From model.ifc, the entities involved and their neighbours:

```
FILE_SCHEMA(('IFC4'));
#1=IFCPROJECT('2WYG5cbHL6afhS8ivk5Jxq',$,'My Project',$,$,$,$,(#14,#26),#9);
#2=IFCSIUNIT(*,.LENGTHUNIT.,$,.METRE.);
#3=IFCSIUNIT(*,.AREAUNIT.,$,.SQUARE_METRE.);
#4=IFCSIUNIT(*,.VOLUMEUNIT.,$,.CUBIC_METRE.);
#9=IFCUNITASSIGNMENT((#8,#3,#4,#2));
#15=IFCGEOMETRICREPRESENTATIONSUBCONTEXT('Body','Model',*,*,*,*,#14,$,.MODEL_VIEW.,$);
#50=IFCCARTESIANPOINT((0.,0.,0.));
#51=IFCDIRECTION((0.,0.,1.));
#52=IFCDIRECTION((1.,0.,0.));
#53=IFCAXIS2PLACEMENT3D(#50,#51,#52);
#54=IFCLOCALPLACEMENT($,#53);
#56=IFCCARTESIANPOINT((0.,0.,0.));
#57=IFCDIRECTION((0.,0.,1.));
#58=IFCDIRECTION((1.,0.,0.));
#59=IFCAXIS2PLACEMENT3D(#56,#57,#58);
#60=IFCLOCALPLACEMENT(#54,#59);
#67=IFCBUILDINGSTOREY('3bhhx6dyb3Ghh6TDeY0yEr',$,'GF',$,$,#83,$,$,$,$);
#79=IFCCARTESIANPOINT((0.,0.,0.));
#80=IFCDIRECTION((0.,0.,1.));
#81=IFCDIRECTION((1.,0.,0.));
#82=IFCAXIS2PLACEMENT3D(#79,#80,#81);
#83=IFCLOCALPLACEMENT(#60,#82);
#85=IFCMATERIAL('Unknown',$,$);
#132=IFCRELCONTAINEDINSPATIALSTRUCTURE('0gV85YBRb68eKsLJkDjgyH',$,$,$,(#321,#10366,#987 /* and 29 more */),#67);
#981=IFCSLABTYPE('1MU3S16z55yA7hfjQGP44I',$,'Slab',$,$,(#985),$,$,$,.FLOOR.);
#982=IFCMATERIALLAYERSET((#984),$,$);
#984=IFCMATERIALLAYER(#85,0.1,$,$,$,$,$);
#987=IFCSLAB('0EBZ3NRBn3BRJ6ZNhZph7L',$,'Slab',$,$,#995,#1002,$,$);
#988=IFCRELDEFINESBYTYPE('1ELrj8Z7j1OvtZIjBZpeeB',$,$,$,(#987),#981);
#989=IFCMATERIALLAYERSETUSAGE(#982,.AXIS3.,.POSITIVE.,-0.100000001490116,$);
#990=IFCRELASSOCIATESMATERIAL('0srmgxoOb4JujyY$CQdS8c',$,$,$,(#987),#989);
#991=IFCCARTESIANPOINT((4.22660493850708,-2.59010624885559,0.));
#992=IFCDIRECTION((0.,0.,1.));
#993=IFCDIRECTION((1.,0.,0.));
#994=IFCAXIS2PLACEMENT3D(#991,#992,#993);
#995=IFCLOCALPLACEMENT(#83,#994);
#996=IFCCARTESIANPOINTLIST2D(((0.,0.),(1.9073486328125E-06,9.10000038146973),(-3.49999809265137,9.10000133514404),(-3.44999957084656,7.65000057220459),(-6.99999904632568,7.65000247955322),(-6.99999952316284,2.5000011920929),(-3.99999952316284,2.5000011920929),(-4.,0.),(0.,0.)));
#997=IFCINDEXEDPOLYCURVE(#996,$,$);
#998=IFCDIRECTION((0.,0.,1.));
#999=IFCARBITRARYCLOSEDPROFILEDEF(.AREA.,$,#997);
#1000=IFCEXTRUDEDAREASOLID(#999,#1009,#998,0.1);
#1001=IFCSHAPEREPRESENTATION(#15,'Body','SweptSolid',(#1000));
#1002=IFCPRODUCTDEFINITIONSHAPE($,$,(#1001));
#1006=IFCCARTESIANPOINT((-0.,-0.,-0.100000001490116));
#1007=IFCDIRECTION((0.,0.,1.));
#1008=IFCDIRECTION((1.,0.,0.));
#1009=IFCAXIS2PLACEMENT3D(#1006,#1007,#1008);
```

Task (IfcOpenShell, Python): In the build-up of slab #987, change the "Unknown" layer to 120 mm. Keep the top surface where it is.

```python
import ifcopenshell
import ifcopenshell.util.element
import ifcopenshell.util.representation

model = ifcopenshell.open("model.ifc")

layer_set = model.by_id(982)
layer = next(l for l in layer_set.MaterialLayers if l.Material and l.Material.Name == "Unknown")
change = 0.12 - layer.LayerThickness
layer.LayerThickness += change

# Geometry does not follow the layer set by itself.
slabs = [e for e in ifcopenshell.util.element.get_elements_by_material(model, layer_set) if e.is_a("IfcSlab")]
for slab in sorted(slabs, key=lambda e: e.id()):
    body = ifcopenshell.util.representation.get_representation(slab, "Model", "Body")
    solid = body.Items[0]
    old_depth = solid.Depth
    solid.Depth += change
    # Extruded upwards: lower the start of the extrusion so the top stays.
    x, y, z = solid.Position.Location.Coordinates
    solid.Position.Location = model.createIfcCartesianPoint((x, y, z - change))
    print(slab.id(), f"{old_depth:g} -> {solid.Depth:g}")

# The layers are counted up from the underside, which has moved.
for usage in {ifcopenshell.util.element.get_material(slab) for slab in slabs}:
    usage.OffsetFromReferenceLine -= change

model.write("model_rev.ifc")
```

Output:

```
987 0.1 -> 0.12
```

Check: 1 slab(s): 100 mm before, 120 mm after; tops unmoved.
